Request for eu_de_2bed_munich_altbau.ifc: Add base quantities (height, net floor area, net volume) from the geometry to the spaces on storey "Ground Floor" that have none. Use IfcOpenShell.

First a look at what the model holds.

```python
import ifcopenshell
import ifcopenshell.util.element
import ifcopenshell.util.unit

model = ifcopenshell.open("eu_de_2bed_munich_altbau.ifc")
print(model.schema)
for unit_type in ("LENGTHUNIT", "AREAUNIT", "VOLUMEUNIT"):
    print(unit_type, ifcopenshell.util.unit.calculate_unit_scale(model, unit_type))
storey = next(s for s in model.by_type("IfcBuildingStorey") if s.Name == "Ground Floor")
spaces = [e for e in ifcopenshell.util.element.get_decomposition(storey) if e.is_a("IfcSpace")]
for e in sorted(spaces, key=lambda e: e.id()):
    print(e.id(), e.is_a(), e.Name, list(ifcopenshell.util.element.get_psets(e, qtos_only=True)), sep=" | ")
```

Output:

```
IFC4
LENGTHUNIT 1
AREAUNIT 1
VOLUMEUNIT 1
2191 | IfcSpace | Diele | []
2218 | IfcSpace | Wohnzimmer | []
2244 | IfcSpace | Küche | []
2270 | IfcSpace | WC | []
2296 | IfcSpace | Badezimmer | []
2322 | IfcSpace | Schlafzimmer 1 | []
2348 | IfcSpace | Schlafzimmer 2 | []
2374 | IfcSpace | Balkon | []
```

```python
import ifcopenshell
import ifcopenshell.api.pset
import ifcopenshell.geom
import ifcopenshell.util.element
import ifcopenshell.util.shape
import ifcopenshell.util.unit

model = ifcopenshell.open("eu_de_2bed_munich_altbau.ifc")
unit_scale = ifcopenshell.util.unit.calculate_unit_scale(model)
area_scale = ifcopenshell.util.unit.calculate_unit_scale(model, "AREAUNIT")
volume_scale = ifcopenshell.util.unit.calculate_unit_scale(model, "VOLUMEUNIT")
settings = ifcopenshell.geom.settings()

storey = next(s for s in model.by_type("IfcBuildingStorey") if s.Name == "Ground Floor")
spaces = [e for e in ifcopenshell.util.element.get_decomposition(storey) if e.is_a("IfcSpace")]

for e in sorted(spaces, key=lambda e: e.id()):
    if ifcopenshell.util.element.get_psets(e, qtos_only=True, should_inherit=False):
        continue
    # Geometry comes back in metres, in the element's own axes.
    shape = ifcopenshell.geom.create_shape(settings, e)
    values = {
        "Height": ifcopenshell.util.shape.get_z(shape.geometry) / unit_scale,
        "NetFloorArea": ifcopenshell.util.shape.get_footprint_area(shape.geometry) / area_scale,
        "NetVolume": ifcopenshell.util.shape.get_volume(shape.geometry) / volume_scale,
    }
    qto = ifcopenshell.api.pset.add_qto(model, product=e, name="Qto_SpaceBaseQuantities")
    ifcopenshell.api.pset.edit_qto(model, qto=qto, properties=values)
    print(e.id(), {k: round(v, 3) for k, v in values.items()})

model.write("eu_de_2bed_munich_altbau_edited.ifc")
```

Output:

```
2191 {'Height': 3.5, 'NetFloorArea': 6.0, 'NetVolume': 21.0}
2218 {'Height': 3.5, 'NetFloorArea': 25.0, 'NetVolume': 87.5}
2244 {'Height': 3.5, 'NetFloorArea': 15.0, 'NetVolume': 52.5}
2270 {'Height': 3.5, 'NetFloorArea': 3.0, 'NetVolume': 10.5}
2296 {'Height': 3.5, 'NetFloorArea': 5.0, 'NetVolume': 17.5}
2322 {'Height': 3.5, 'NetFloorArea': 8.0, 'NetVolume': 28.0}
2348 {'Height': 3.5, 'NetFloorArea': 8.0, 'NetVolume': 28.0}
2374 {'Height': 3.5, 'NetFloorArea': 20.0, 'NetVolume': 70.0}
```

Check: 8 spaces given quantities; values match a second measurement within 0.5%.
